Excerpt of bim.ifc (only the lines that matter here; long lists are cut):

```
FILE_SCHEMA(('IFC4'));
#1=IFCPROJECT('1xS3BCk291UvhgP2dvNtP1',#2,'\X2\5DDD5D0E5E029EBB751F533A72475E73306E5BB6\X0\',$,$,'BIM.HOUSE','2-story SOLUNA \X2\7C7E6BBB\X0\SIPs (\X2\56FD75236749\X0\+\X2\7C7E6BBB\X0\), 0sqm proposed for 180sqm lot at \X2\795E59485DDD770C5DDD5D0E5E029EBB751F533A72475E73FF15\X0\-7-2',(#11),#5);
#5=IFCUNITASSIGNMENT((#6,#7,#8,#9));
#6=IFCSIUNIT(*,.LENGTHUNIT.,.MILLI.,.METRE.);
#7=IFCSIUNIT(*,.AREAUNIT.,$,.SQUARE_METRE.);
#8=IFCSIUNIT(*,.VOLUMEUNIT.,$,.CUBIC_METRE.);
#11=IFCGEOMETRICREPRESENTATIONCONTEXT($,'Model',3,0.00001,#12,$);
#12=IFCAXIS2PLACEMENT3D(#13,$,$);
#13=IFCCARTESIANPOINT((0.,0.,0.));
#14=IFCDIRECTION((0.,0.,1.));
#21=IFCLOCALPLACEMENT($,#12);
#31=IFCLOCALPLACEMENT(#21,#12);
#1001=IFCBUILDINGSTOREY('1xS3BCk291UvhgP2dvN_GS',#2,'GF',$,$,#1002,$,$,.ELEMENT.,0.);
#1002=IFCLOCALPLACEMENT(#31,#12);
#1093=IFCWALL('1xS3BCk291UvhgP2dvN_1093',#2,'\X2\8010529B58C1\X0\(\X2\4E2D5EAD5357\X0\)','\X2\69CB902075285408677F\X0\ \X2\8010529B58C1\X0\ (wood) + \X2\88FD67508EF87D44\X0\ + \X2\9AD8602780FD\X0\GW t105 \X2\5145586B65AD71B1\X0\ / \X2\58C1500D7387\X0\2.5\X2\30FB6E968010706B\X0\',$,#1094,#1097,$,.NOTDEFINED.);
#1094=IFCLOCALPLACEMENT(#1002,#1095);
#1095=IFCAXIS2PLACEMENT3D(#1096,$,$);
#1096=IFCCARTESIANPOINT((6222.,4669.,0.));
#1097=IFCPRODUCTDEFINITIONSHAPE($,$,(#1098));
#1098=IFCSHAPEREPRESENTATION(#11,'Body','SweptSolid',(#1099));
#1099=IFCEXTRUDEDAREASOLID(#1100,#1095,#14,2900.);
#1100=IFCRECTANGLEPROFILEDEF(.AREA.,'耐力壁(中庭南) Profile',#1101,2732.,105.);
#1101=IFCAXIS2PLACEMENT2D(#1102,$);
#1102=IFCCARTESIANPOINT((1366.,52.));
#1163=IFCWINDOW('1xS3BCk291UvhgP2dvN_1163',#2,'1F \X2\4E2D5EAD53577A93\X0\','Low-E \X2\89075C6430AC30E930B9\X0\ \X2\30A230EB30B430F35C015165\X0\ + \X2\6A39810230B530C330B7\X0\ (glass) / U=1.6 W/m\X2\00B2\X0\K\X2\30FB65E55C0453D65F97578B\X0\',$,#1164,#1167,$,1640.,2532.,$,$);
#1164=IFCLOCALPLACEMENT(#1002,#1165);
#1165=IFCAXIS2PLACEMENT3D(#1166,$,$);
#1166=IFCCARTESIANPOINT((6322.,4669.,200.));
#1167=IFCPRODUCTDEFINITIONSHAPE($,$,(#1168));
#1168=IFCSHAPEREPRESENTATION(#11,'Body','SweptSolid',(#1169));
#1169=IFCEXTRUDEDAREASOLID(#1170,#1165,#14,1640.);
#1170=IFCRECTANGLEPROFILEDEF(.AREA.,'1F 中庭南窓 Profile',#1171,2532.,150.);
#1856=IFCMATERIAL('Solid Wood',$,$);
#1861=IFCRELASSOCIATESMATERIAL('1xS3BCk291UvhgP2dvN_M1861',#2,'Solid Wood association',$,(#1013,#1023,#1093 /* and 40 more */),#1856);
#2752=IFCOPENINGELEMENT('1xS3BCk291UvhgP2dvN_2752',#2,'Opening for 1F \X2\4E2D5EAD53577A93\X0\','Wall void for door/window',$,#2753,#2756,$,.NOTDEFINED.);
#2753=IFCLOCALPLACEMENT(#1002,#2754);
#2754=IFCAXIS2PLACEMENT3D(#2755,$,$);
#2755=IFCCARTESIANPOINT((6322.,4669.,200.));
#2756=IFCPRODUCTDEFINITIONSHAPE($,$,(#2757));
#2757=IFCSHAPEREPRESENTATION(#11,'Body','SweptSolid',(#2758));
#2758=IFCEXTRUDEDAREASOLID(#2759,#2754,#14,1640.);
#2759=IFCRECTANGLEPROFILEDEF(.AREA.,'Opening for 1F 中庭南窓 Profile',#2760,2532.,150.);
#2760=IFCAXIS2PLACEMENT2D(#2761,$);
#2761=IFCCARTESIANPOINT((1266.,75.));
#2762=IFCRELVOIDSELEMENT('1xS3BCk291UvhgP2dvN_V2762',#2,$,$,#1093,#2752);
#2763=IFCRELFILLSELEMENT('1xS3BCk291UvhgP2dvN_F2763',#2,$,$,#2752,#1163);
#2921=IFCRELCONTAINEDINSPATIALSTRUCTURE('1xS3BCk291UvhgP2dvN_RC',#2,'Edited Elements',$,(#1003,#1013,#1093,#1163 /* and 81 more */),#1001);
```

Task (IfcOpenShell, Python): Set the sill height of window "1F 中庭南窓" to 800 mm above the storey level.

```python
import numpy as np
import ifcopenshell
import ifcopenshell.api.geometry
import ifcopenshell.geom
import ifcopenshell.util.element
import ifcopenshell.util.placement
import ifcopenshell.util.shape
import ifcopenshell.util.unit

model = ifcopenshell.open("bim.ifc")
unit_scale = ifcopenshell.util.unit.calculate_unit_scale(model)

window = model.by_guid("1xS3BCk291UvhgP2dvN_1163")
opening = window.FillsVoids[0].RelatingOpeningElement
storey = ifcopenshell.util.element.get_container(window, ifc_class="IfcBuildingStorey")
level = ifcopenshell.util.placement.get_local_placement(storey.ObjectPlacement)[2, 3]

# The opening's origin need not be at the sill, so measure its lowest point.
shape = ifcopenshell.geom.create_shape(ifcopenshell.geom.settings(), opening)
bottom = ifcopenshell.util.shape.get_shape_bottom_elevation(shape, shape.geometry) / unit_scale
dz = level + 800.0 - bottom

shift = np.array([0.0, 0.0, dz])
# The window is not placed relative to its opening, so move both.
for product in (opening, window):
    matrix = ifcopenshell.util.placement.get_local_placement(product.ObjectPlacement)
    matrix[:3, 3] += shift
    ifcopenshell.api.geometry.edit_object_placement(model, product=product, matrix=matrix, is_si=False)

print(f"moved by {dz * unit_scale:+.3f} m")

model.write("bim_v2.ifc")
```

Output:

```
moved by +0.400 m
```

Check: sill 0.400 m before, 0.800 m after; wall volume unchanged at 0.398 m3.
